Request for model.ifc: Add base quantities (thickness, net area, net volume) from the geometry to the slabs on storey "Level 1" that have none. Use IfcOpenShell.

First a look at what the model holds.

```python
import ifcopenshell
import ifcopenshell.util.element
import ifcopenshell.util.unit

model = ifcopenshell.open("model.ifc")
print(model.schema)
for unit_type in ("LENGTHUNIT", "AREAUNIT", "VOLUMEUNIT"):
    print(unit_type, ifcopenshell.util.unit.calculate_unit_scale(model, unit_type))
storey = next(s for s in model.by_type("IfcBuildingStorey") if s.Name == "Level 1")
slabs = [e for e in ifcopenshell.util.element.get_decomposition(storey) if e.is_a("IfcSlab")]
for e in sorted(slabs, key=lambda e: e.id()):
    print(e.id(), e.is_a(), e.Name, list(ifcopenshell.util.element.get_psets(e, qtos_only=True)), sep=" | ")
```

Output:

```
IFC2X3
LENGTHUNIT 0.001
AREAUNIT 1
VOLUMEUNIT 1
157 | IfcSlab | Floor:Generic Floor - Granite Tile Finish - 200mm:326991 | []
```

```python
import ifcopenshell
import ifcopenshell.api.pset
import ifcopenshell.geom
import ifcopenshell.util.element
import ifcopenshell.util.shape
import ifcopenshell.util.unit

model = ifcopenshell.open("model.ifc")
unit_scale = ifcopenshell.util.unit.calculate_unit_scale(model)
area_scale = ifcopenshell.util.unit.calculate_unit_scale(model, "AREAUNIT")
volume_scale = ifcopenshell.util.unit.calculate_unit_scale(model, "VOLUMEUNIT")
settings = ifcopenshell.geom.settings()

storey = next(s for s in model.by_type("IfcBuildingStorey") if s.Name == "Level 1")
slabs = [e for e in ifcopenshell.util.element.get_decomposition(storey) if e.is_a("IfcSlab")]

for e in sorted(slabs, key=lambda e: e.id()):
    if ifcopenshell.util.element.get_psets(e, qtos_only=True, should_inherit=False):
        continue
    # Geometry comes back in metres, in the element's own axes.
    shape = ifcopenshell.geom.create_shape(settings, e)
    values = {
        "Width": ifcopenshell.util.shape.get_z(shape.geometry) / unit_scale,
        "NetArea": ifcopenshell.util.shape.get_footprint_area(shape.geometry) / area_scale,
        "NetVolume": ifcopenshell.util.shape.get_volume(shape.geometry) / volume_scale,
    }
    qto = ifcopenshell.api.pset.add_qto(model, product=e, name="BaseQuantities")
    ifcopenshell.api.pset.edit_qto(model, qto=qto, properties=values)
    print(e.id(), {k: round(v, 3) for k, v in values.items()})

model.write("model-out.ifc")
```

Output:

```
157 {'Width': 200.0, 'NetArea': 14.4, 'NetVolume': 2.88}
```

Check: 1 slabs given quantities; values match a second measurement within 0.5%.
